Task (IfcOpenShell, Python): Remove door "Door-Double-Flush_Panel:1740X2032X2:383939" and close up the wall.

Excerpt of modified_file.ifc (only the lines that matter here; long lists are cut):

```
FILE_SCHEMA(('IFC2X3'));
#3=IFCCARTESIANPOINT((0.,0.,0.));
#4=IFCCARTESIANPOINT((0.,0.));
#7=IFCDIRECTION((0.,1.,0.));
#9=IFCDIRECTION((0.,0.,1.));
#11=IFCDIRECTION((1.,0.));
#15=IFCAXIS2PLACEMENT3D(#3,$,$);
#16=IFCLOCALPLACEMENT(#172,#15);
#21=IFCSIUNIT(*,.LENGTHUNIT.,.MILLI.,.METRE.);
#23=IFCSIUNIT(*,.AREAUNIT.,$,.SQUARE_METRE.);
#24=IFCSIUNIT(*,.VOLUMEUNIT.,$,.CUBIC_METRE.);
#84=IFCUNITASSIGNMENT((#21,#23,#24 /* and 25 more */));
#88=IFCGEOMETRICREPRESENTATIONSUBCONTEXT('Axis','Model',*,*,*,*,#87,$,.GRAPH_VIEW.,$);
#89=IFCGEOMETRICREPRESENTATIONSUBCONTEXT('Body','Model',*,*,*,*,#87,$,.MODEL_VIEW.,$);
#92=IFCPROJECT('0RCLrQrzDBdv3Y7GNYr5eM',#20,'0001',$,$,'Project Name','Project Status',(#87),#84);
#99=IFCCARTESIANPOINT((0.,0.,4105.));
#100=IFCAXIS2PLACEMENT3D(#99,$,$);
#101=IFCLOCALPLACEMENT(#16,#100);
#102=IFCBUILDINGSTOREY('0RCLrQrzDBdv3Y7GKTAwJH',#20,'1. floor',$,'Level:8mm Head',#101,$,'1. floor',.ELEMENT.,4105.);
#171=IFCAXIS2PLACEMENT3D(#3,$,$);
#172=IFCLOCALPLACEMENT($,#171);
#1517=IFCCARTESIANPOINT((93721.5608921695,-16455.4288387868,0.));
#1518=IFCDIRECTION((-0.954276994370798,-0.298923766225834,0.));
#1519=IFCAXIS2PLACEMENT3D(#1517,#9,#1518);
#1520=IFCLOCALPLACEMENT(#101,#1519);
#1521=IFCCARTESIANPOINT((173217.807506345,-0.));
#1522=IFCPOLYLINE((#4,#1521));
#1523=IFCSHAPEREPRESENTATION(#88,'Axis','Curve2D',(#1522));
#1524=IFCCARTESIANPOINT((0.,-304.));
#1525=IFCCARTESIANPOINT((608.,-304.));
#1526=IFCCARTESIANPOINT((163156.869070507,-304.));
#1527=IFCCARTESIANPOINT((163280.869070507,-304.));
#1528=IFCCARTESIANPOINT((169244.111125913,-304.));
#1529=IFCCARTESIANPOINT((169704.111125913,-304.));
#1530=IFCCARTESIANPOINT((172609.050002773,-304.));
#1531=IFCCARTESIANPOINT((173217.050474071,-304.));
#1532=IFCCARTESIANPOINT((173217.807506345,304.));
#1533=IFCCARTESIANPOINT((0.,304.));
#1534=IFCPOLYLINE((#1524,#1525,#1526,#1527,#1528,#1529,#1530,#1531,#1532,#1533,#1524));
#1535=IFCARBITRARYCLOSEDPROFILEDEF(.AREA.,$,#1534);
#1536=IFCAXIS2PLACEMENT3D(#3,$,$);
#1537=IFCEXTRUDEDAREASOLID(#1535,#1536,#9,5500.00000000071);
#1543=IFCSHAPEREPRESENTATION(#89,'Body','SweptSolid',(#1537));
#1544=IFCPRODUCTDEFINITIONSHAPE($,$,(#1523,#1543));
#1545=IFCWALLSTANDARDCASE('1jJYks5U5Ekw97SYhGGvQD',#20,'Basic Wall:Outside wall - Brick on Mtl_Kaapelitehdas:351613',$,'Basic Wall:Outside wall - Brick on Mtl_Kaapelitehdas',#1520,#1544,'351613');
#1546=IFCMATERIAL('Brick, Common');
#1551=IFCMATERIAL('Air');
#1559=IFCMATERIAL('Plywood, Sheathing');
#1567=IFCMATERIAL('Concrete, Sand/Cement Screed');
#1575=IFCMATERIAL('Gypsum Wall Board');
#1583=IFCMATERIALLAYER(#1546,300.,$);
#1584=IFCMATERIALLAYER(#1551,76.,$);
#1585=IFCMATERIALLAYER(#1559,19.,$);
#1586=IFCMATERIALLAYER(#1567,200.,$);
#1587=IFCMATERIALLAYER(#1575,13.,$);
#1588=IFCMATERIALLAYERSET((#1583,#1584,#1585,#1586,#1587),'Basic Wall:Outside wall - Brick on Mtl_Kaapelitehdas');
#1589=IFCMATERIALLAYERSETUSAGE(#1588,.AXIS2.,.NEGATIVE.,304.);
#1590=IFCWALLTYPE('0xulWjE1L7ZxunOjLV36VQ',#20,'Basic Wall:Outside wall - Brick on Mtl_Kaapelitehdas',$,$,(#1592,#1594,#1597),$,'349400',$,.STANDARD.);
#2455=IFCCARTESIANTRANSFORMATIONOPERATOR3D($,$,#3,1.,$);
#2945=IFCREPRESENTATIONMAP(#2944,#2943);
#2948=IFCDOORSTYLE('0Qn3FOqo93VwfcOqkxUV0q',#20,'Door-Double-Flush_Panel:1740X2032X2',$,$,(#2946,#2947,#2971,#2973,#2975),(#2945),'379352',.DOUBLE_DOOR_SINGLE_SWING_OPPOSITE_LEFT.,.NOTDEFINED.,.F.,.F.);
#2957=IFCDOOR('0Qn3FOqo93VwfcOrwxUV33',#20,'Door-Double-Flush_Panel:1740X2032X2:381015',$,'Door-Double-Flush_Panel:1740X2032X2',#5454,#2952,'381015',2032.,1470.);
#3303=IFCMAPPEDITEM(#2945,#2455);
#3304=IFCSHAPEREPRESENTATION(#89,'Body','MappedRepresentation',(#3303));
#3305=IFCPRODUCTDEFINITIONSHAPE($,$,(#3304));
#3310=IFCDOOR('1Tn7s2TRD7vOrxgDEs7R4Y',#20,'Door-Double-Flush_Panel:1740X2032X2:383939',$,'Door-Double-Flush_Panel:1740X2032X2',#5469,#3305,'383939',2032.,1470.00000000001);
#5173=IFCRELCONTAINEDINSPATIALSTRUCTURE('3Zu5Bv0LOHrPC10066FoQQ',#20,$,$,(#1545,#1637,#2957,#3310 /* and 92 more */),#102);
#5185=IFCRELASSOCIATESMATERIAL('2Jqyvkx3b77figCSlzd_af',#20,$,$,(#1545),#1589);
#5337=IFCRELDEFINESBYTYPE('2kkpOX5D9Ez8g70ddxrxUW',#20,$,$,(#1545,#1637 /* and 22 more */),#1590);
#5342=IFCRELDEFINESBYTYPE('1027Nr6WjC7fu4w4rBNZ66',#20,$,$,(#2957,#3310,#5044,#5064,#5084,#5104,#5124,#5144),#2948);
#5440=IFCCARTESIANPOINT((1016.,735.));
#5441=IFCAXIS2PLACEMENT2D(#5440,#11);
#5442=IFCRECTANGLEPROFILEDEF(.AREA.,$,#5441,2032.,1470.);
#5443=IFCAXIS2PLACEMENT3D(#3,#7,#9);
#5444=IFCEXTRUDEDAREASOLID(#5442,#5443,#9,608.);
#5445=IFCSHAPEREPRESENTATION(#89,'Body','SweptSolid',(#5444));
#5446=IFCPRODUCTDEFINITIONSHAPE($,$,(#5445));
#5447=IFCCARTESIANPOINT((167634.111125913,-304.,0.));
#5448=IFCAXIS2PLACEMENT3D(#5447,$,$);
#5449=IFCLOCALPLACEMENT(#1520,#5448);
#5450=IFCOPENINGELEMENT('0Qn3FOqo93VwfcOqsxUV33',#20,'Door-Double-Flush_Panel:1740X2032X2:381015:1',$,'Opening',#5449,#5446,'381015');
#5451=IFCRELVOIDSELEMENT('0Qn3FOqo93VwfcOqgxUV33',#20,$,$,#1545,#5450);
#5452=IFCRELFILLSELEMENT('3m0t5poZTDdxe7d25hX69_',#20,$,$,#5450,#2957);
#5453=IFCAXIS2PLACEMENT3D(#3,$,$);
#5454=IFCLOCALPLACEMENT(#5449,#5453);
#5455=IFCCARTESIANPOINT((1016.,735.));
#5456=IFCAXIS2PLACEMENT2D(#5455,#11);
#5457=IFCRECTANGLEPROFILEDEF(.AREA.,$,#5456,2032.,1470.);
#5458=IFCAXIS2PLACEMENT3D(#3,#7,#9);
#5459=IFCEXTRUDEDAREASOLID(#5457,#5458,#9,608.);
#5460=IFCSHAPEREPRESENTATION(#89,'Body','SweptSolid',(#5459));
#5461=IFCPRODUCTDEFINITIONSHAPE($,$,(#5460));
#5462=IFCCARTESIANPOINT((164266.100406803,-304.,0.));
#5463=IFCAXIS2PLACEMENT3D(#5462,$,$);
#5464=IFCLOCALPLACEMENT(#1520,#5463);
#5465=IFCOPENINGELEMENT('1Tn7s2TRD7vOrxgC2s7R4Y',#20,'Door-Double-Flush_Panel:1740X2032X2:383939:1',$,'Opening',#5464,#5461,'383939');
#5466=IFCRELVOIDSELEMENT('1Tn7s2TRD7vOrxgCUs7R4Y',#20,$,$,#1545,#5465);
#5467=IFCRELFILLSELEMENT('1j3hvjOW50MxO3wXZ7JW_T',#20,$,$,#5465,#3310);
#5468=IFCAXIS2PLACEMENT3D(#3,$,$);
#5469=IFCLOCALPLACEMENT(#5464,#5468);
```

```python
import ifcopenshell
import ifcopenshell.api.feature
import ifcopenshell.api.root
import ifcopenshell.geom
import ifcopenshell.util.shape

model = ifcopenshell.open("modified_file.ifc")
settings = ifcopenshell.geom.settings()


def volume(element):
    """Net volume in cubic metres, openings subtracted."""
    shape = ifcopenshell.geom.create_shape(settings, element)
    return ifcopenshell.util.shape.get_volume(shape.geometry)


door = model.by_guid("1Tn7s2TRD7vOrxgDEs7R4Y")
opening = door.FillsVoids[0].RelatingOpeningElement
wall = opening.VoidsElements[0].RelatingBuildingElement
before = volume(wall)

ifcopenshell.api.root.remove_product(model, product=door)
ifcopenshell.api.feature.remove_feature(model, feature=opening)

after = volume(wall)

print(f"wall volume {before:.3f} -> {after:.3f} m3")

model.write("modified_file_edited.ifc")
```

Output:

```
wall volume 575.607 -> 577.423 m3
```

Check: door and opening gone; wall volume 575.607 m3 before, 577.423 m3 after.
